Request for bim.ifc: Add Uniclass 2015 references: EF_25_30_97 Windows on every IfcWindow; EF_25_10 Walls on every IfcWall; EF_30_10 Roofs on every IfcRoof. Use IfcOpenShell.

First a look at what the model holds.

```python
import ifcopenshell

model = ifcopenshell.open("bim.ifc")
print(model.schema)
print("classifications:", [c.Name for c in model.by_type("IfcClassification")])
for ifc_class in ("IfcDoor", "IfcRoof", "IfcStair", "IfcWall", "IfcWindow"):
    print(ifc_class, len(model.by_type(ifc_class)))
```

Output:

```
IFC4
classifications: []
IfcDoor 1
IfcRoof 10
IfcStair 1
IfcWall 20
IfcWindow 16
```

```python
import ifcopenshell
import ifcopenshell.api.classification

model = ifcopenshell.open("bim.ifc")

system = ifcopenshell.api.classification.add_classification(model, classification="Uniclass 2015")

codes = {
    "IfcWindow": ("EF_25_30_97", "Windows"),
    "IfcWall": ("EF_25_10", "Walls"),
    "IfcRoof": ("EF_30_10", "Roofs"),
}
for ifc_class, (code, name) in codes.items():
    products = model.by_type(ifc_class)
    ifcopenshell.api.classification.add_reference(
        model, products=products, classification=system, identification=code, name=name
    )
    print(code, len(products))

model.write("bim_updated.ifc")
```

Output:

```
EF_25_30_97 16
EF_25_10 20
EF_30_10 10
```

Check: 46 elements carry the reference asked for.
